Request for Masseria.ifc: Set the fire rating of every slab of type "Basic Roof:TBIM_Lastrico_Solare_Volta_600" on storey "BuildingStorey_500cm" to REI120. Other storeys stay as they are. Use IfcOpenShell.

First a look at what the model holds.

```python
import ifcopenshell
import ifcopenshell.util.element

model = ifcopenshell.open("Masseria.ifc")
print(model.schema)
storey = next(s for s in model.by_type("IfcBuildingStorey") if s.Name == "BuildingStorey_500cm")
slabs = [e for e in ifcopenshell.util.element.get_decomposition(storey) if e.is_a("IfcSlab")]
seen = {}
for e in slabs:
    element_type = ifcopenshell.util.element.get_type(e)
    key = (element_type.Name if element_type != e and element_type else None, ifcopenshell.util.element.get_pset(e, "Pset_SlabCommon", "FireRating"))
    seen[key] = seen.get(key, 0) + 1
for (name, value), count in sorted(seen.items(), key=str):
    print(count, "x", name, "|", value)
```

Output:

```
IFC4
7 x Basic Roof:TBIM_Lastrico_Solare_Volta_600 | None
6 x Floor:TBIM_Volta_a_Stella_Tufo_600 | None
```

```python
import ifcopenshell
import ifcopenshell.api.pset
import ifcopenshell.util.element

model = ifcopenshell.open("Masseria.ifc")

storey = next(s for s in model.by_type("IfcBuildingStorey") if s.Name == "BuildingStorey_500cm")
slabs = [e for e in ifcopenshell.util.element.get_decomposition(storey) if e.is_a("IfcSlab")]

count = 0
for e in slabs:
    element_type = ifcopenshell.util.element.get_type(e)
    if element_type in (None, e) or element_type.Name != "Basic Roof:TBIM_Lastrico_Solare_Volta_600":
        continue
    # add_pset returns the element's existing set when there is one.
    pset = ifcopenshell.api.pset.add_pset(model, product=e, name="Pset_SlabCommon")
    ifcopenshell.api.pset.edit_pset(model, pset=pset, properties={"FireRating": "REI120"})
    count += 1

print(count, "slabs updated")

model.write("Masseria_edited.ifc")
```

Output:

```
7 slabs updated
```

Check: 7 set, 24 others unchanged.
